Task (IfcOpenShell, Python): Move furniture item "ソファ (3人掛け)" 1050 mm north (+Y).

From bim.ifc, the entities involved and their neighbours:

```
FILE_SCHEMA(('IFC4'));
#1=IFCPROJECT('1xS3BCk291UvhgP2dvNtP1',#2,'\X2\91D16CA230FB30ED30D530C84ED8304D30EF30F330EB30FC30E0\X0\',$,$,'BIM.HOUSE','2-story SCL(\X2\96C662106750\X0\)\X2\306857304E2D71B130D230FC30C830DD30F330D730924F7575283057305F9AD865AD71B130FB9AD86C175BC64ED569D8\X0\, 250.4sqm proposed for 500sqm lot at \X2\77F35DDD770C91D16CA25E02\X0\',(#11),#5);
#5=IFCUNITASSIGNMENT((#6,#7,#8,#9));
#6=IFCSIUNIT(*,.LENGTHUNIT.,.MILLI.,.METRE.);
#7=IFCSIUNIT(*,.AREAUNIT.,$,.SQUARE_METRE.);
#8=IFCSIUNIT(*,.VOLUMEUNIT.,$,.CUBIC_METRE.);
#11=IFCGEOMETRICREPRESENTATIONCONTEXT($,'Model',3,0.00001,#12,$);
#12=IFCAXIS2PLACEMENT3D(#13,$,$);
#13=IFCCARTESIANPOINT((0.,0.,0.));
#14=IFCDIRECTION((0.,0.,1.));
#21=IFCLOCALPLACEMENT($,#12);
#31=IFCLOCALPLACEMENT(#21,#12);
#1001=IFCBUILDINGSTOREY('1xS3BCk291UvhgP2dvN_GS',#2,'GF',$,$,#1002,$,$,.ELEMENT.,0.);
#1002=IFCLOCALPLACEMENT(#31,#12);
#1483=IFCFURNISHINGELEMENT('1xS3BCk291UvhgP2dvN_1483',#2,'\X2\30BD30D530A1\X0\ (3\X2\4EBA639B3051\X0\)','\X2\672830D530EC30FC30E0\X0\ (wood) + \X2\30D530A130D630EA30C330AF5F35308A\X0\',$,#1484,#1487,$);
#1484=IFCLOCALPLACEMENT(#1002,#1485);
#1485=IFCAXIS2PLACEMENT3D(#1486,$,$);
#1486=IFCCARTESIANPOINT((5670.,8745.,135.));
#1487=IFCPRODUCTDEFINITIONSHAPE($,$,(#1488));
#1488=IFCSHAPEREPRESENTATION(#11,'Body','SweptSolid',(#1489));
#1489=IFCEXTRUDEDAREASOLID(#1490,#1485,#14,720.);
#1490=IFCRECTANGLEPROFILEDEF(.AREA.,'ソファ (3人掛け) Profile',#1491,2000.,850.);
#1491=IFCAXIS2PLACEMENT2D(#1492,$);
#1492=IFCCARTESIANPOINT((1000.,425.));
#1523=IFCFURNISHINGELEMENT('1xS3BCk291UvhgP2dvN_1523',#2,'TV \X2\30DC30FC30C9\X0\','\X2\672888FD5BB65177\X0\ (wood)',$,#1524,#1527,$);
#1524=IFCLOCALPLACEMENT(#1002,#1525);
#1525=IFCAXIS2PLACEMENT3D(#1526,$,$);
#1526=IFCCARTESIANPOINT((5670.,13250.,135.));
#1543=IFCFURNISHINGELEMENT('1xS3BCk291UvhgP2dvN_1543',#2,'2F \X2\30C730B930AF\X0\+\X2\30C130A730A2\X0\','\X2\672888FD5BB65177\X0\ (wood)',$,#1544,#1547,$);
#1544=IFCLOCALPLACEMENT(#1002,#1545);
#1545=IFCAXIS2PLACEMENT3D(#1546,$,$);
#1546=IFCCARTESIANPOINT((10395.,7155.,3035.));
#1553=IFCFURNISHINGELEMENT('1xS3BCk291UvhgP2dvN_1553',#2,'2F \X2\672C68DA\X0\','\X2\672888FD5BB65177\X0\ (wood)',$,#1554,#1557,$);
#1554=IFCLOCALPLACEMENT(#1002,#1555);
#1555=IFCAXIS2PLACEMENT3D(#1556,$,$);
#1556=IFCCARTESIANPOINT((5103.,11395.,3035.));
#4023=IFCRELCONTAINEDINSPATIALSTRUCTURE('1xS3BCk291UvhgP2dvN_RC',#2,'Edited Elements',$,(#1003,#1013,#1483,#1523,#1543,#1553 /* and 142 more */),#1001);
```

```python
import ifcopenshell
import ifcopenshell.api.geometry
import ifcopenshell.util.placement
import ifcopenshell.util.unit

model = ifcopenshell.open("bim.ifc")
unit_scale = ifcopenshell.util.unit.calculate_unit_scale(model)

item = model.by_id(1483)
matrix = ifcopenshell.util.placement.get_local_placement(item.ObjectPlacement)
matrix[1, 3] += 1.05 / unit_scale
ifcopenshell.api.geometry.edit_object_placement(model, product=item, matrix=matrix, is_si=False)

print(ifcopenshell.util.placement.get_local_placement(item.ObjectPlacement).round(3) + 0.0)

model.write("bim_edited.ifc")
```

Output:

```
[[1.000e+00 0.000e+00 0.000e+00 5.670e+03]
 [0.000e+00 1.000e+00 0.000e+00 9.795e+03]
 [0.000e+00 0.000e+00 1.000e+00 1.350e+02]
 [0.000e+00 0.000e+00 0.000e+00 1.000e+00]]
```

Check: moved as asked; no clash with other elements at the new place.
